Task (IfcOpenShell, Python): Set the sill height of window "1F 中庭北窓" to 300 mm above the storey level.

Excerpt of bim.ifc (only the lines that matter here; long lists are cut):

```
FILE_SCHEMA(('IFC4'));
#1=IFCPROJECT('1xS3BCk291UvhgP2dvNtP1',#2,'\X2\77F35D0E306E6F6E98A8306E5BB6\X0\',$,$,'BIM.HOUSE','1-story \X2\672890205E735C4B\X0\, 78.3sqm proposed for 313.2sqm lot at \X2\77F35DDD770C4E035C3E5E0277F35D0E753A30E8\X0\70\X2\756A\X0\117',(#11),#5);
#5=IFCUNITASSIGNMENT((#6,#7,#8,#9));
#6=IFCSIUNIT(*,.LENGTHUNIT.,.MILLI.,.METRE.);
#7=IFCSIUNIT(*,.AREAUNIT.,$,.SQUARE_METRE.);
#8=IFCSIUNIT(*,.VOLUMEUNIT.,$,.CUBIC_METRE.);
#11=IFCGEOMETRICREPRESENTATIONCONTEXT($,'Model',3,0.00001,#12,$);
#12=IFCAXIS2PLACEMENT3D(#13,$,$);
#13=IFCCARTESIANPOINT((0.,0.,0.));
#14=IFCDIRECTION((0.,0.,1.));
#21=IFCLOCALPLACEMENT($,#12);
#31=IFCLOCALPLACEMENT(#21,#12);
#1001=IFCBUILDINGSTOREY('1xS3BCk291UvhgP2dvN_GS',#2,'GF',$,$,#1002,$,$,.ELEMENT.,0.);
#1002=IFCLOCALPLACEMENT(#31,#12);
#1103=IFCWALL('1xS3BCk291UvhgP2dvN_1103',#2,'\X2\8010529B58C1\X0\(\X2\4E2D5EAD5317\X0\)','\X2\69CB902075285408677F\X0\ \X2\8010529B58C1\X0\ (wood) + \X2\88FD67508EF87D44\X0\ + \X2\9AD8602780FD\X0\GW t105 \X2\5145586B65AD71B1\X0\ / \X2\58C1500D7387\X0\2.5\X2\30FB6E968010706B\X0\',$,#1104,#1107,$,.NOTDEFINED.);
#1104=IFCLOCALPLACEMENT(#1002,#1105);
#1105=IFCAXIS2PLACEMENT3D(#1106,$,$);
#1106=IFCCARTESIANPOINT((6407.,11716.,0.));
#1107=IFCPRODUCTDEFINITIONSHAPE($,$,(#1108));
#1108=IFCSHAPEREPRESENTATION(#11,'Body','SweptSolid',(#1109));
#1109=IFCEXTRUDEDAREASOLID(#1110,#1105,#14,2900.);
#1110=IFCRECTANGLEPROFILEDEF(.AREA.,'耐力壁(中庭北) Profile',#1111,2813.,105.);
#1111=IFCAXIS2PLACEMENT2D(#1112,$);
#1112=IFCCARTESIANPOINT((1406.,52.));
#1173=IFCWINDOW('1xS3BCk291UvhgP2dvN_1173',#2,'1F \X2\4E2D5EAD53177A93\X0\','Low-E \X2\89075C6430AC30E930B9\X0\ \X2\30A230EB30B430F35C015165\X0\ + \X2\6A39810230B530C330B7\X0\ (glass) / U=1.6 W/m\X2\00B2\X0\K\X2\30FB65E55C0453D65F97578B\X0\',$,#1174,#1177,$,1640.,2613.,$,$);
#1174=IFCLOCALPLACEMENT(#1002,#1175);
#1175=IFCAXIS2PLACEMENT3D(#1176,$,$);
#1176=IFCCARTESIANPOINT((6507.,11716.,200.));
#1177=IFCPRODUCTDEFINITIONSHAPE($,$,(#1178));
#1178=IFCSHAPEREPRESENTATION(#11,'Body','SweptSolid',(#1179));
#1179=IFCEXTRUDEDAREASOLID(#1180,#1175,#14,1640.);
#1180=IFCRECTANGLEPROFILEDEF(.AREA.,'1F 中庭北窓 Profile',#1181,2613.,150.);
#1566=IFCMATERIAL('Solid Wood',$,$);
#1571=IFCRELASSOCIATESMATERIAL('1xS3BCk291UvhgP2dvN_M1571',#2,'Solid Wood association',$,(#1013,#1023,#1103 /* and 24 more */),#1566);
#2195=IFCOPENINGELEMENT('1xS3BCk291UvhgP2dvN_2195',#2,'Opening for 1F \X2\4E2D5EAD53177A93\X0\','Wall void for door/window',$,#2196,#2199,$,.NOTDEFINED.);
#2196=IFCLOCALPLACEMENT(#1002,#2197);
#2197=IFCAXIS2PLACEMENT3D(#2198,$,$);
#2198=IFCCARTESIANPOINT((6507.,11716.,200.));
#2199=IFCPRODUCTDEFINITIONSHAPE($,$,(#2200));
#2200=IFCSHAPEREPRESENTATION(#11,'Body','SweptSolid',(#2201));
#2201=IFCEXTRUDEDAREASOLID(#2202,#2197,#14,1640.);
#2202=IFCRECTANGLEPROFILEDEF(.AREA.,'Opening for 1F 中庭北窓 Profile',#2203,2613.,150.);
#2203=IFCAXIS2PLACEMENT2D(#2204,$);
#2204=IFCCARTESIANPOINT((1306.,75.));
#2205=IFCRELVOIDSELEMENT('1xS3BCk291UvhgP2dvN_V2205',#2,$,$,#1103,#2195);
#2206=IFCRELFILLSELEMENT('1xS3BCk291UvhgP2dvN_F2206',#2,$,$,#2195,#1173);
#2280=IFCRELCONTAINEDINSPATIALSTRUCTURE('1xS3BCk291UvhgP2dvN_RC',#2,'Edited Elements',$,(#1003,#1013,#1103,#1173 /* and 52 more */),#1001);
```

```python
import numpy as np
import ifcopenshell
import ifcopenshell.api.geometry
import ifcopenshell.geom
import ifcopenshell.util.element
import ifcopenshell.util.placement
import ifcopenshell.util.shape
import ifcopenshell.util.unit

model = ifcopenshell.open("bim.ifc")
unit_scale = ifcopenshell.util.unit.calculate_unit_scale(model)

window = model.by_id(1173)
opening = window.FillsVoids[0].RelatingOpeningElement
storey = ifcopenshell.util.element.get_container(window, ifc_class="IfcBuildingStorey")
level = ifcopenshell.util.placement.get_local_placement(storey.ObjectPlacement)[2, 3]

# The opening's origin need not be at the sill, so measure its lowest point.
shape = ifcopenshell.geom.create_shape(ifcopenshell.geom.settings(), opening)
bottom = ifcopenshell.util.shape.get_shape_bottom_elevation(shape, shape.geometry) / unit_scale
dz = level + 0.3 / unit_scale - bottom

shift = np.array([0.0, 0.0, dz])
# The window is not placed relative to its opening, so move both.
for product in (opening, window):
    matrix = ifcopenshell.util.placement.get_local_placement(product.ObjectPlacement)
    matrix[:3, 3] += shift
    ifcopenshell.api.geometry.edit_object_placement(model, product=product, matrix=matrix, is_si=False)

print(f"moved by {dz * unit_scale:+.3f} m")

model.write("bim_rev.ifc")
```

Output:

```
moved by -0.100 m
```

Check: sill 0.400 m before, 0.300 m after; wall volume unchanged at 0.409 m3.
